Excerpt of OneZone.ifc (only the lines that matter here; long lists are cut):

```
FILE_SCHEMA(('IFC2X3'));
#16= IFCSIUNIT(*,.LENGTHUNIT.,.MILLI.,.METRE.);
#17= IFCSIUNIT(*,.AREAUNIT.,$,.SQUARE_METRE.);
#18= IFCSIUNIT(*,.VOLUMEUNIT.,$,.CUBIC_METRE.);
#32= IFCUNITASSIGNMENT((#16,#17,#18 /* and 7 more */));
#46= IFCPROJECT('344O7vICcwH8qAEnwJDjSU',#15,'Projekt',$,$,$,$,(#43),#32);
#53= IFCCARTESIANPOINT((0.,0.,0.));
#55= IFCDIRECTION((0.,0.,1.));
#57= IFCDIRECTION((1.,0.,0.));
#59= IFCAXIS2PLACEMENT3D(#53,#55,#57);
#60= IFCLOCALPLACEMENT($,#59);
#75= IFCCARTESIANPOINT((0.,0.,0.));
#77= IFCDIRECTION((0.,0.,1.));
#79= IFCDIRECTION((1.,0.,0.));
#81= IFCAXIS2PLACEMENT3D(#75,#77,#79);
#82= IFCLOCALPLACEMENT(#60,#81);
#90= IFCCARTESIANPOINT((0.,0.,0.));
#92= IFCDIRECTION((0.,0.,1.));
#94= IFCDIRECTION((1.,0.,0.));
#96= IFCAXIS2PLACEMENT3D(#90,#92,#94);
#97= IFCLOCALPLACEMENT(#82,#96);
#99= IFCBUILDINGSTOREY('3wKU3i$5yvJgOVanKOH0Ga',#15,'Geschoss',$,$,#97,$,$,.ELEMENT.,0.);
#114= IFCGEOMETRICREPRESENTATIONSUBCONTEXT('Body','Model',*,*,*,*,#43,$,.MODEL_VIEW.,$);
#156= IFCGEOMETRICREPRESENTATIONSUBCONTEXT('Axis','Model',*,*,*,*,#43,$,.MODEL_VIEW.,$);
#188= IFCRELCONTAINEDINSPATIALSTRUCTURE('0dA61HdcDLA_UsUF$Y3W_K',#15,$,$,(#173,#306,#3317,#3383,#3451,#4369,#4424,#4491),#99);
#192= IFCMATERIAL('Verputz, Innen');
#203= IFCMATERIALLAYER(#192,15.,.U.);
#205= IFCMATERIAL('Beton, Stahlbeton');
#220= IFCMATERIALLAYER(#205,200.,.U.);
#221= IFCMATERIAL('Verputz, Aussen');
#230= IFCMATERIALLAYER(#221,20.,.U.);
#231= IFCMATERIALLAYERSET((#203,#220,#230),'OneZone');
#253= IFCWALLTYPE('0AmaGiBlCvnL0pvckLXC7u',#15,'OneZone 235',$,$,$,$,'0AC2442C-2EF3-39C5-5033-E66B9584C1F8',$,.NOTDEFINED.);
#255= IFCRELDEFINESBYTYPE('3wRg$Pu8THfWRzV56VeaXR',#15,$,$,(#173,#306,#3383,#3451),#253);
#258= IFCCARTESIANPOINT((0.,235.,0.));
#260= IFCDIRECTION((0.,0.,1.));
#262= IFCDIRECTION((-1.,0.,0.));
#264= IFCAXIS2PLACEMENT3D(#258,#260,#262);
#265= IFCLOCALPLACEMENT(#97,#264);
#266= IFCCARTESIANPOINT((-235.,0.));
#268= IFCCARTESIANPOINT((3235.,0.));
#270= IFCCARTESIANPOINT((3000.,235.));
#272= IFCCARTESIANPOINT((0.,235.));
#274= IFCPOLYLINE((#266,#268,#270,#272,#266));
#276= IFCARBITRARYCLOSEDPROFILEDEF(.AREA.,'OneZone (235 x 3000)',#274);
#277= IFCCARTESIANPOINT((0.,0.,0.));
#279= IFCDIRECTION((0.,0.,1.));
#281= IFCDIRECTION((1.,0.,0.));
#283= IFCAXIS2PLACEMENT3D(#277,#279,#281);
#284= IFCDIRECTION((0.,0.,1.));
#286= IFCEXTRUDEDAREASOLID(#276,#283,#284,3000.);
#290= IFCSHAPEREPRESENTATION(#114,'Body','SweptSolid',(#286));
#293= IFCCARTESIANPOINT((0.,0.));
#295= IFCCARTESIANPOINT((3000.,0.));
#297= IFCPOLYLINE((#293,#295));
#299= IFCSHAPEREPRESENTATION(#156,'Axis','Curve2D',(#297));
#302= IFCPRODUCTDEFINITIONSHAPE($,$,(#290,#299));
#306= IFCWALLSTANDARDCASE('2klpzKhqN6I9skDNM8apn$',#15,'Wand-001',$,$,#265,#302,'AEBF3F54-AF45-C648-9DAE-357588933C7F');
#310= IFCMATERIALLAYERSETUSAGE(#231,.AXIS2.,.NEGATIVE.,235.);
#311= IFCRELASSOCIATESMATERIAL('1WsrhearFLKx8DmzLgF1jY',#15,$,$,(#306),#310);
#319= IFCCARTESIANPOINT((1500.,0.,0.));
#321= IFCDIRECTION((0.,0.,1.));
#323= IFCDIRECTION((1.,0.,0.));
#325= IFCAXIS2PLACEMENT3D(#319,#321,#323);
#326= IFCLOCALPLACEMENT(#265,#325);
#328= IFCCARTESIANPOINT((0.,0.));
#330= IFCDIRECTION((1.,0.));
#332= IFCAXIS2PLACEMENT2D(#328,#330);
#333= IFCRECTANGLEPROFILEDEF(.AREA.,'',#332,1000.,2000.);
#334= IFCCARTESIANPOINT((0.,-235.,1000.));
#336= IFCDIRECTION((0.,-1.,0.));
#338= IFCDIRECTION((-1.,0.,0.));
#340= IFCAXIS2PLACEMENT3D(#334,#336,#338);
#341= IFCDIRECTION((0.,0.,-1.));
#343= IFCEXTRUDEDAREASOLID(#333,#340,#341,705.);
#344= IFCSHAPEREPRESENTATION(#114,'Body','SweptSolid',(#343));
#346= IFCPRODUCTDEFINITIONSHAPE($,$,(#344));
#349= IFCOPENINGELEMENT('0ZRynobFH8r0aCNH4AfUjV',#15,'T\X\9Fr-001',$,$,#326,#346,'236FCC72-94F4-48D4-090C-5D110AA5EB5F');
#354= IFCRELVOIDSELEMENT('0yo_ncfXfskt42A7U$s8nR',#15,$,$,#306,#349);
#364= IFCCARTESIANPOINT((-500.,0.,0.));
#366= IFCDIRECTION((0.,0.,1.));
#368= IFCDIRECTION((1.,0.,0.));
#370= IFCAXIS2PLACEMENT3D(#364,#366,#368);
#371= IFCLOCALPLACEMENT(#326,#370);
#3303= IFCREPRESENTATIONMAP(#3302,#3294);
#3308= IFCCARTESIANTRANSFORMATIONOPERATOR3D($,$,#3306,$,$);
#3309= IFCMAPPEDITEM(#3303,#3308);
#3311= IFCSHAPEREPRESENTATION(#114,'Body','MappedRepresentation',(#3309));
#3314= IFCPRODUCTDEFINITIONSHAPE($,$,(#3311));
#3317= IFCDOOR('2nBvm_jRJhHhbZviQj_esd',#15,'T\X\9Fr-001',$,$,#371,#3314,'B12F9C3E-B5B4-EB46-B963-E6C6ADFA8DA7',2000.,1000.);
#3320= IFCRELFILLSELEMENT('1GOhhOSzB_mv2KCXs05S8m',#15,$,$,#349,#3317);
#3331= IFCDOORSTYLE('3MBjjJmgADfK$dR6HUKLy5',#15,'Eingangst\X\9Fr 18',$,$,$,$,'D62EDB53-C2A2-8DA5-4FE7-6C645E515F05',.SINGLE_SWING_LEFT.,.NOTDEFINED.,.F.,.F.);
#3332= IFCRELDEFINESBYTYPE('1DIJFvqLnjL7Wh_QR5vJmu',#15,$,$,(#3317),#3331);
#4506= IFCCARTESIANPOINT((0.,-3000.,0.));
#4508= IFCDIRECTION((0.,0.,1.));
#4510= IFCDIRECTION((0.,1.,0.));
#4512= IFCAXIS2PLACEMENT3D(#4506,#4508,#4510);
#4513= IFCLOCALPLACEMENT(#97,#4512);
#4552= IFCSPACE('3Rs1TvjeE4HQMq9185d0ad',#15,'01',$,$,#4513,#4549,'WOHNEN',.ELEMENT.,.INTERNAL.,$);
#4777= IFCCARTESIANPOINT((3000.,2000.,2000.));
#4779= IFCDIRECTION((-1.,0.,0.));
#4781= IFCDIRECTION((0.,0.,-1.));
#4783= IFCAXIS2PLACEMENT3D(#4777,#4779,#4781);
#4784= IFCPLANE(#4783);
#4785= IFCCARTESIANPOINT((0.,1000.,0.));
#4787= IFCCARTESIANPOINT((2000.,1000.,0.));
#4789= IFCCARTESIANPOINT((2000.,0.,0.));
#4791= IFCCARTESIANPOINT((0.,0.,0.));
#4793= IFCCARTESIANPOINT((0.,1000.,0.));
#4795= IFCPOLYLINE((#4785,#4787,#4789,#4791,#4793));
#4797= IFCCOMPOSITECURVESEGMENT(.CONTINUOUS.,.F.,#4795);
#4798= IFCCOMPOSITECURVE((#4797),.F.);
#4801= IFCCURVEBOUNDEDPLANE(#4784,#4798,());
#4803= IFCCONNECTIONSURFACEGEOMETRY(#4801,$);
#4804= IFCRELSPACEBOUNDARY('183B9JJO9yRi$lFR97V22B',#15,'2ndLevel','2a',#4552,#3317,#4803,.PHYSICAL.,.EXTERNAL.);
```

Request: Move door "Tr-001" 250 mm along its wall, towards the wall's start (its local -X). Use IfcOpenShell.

```python
import numpy as np
import ifcopenshell
import ifcopenshell.api.geometry
import ifcopenshell.util.placement

model = ifcopenshell.open("OneZone.ifc")

door = model.by_guid("2nBvm_jRJhHhbZviQj_esd")
opening = door.FillsVoids[0].RelatingOpeningElement
wall = opening.VoidsElements[0].RelatingBuildingElement

wall_matrix = ifcopenshell.util.placement.get_local_placement(wall.ObjectPlacement)
shift = wall_matrix[:3, 0] * -250.0
before = ifcopenshell.util.placement.get_local_placement(door.ObjectPlacement)[:3, 3].copy()

# The door is placed relative to its opening, so it follows when the opening moves.
matrix = ifcopenshell.util.placement.get_local_placement(opening.ObjectPlacement)
matrix[:3, 3] += shift
ifcopenshell.api.geometry.edit_object_placement(
    model, product=opening, matrix=matrix, is_si=False, should_transform_children=True
)

# Space boundary surfaces are stored in each space's coordinates; move them too.
for rel in door.ProvidesBoundaries:
    if not rel.ConnectionGeometry:
        continue
    surface = rel.ConnectionGeometry.SurfaceOnRelatingElement.BasisSurface
    space_matrix = ifcopenshell.util.placement.get_local_placement(rel.RelatingSpace.ObjectPlacement)
    point = np.array(surface.Position.Location.Coordinates) + space_matrix[:3, :3].T @ shift
    surface.Position = model.createIfcAxis2Placement3D(
        model.createIfcCartesianPoint(point.tolist()), surface.Position.Axis, surface.Position.RefDirection
    )

after = ifcopenshell.util.placement.get_local_placement(door.ObjectPlacement)[:3, 3]
print("door moved by", (after - before).round(3) + 0.0)

model.write("OneZone-out.ifc")
```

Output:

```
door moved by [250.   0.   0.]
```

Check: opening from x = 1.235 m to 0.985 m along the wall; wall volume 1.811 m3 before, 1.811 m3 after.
